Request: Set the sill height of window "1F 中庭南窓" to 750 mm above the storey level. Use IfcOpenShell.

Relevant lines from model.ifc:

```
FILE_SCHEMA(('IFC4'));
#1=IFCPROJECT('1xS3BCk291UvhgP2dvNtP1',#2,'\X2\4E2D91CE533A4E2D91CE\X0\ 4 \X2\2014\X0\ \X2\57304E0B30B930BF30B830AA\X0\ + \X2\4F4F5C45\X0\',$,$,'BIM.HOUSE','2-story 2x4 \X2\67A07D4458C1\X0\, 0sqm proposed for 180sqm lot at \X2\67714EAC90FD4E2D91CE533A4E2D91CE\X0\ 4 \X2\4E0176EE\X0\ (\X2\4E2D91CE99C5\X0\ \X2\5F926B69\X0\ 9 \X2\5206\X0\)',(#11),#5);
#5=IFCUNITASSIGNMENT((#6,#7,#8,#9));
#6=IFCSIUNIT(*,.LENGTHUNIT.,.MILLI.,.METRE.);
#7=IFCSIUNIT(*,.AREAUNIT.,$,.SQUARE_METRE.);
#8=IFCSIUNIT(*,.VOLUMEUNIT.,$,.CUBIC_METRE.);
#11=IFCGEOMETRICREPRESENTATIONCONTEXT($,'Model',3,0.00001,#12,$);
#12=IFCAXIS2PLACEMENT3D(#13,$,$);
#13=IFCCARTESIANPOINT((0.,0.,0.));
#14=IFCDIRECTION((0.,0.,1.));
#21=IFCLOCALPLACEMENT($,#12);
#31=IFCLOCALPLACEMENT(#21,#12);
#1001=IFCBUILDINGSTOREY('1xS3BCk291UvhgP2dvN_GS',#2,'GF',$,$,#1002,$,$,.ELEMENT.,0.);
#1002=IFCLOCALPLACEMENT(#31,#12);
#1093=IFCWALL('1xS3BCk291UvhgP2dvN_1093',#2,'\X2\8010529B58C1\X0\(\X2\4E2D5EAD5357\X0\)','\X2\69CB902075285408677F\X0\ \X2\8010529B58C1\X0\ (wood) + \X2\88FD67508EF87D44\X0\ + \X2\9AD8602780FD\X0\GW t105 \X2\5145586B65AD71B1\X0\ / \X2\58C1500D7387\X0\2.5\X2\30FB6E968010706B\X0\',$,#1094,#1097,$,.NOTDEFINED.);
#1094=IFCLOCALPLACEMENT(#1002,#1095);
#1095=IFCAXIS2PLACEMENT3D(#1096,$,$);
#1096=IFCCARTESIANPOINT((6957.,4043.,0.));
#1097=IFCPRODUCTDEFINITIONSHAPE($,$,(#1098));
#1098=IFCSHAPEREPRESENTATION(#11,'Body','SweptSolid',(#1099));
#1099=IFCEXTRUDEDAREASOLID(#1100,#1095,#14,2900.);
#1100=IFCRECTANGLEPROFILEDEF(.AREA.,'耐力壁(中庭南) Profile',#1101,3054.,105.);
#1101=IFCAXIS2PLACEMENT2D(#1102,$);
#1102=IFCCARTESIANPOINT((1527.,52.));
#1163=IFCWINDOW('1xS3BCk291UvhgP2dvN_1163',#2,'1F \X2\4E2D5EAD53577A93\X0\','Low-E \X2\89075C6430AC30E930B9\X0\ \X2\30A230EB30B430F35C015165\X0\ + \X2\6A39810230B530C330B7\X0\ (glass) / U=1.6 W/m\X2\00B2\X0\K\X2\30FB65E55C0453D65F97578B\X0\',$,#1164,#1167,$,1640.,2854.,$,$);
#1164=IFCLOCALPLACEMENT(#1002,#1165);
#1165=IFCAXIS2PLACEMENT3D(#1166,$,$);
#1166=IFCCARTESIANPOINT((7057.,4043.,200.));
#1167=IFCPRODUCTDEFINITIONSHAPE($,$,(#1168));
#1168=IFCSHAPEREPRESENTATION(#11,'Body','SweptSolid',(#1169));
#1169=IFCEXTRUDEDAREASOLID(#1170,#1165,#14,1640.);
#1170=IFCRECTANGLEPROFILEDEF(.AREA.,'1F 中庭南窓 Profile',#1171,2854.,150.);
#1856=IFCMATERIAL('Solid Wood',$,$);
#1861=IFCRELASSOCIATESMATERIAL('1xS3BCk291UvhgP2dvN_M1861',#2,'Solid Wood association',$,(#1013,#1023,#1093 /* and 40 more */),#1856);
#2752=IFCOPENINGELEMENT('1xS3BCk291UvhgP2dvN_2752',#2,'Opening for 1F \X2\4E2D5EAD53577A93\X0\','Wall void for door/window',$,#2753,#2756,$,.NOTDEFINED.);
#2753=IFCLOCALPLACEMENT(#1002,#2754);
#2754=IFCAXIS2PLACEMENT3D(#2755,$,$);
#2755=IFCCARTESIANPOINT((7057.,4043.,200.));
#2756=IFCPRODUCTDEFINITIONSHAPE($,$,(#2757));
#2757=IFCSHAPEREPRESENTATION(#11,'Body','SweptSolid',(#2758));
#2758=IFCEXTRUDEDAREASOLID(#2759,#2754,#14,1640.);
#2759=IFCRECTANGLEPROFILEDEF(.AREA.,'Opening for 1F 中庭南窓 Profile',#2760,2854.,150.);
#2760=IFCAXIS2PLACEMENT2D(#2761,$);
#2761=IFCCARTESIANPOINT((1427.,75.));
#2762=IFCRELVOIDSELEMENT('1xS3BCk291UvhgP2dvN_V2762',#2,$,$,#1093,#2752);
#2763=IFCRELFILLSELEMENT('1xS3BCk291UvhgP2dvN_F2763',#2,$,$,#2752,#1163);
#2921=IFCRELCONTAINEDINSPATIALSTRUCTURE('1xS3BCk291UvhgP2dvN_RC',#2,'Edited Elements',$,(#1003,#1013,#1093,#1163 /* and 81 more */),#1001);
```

```python
import numpy as np
import ifcopenshell
import ifcopenshell.api.geometry
import ifcopenshell.geom
import ifcopenshell.util.element
import ifcopenshell.util.placement
import ifcopenshell.util.shape
import ifcopenshell.util.unit

model = ifcopenshell.open("model.ifc")
unit_scale = ifcopenshell.util.unit.calculate_unit_scale(model)

window = model.by_id(1163)
opening = window.FillsVoids[0].RelatingOpeningElement
storey = ifcopenshell.util.element.get_container(window, ifc_class="IfcBuildingStorey")
level = ifcopenshell.util.placement.get_local_placement(storey.ObjectPlacement)[2, 3]

# The opening's origin need not be at the sill, so measure its lowest point.
shape = ifcopenshell.geom.create_shape(ifcopenshell.geom.settings(), opening)
bottom = ifcopenshell.util.shape.get_shape_bottom_elevation(shape, shape.geometry) / unit_scale
dz = level + 0.75 / unit_scale - bottom

shift = np.array([0.0, 0.0, dz])
# The window is not placed relative to its opening, so move both.
for product in (opening, window):
    matrix = ifcopenshell.util.placement.get_local_placement(product.ObjectPlacement)
    matrix[:3, 3] += shift
    ifcopenshell.api.geometry.edit_object_placement(model, product=product, matrix=matrix, is_si=False)

print(f"moved by {dz * unit_scale:+.3f} m")

model.write("model_v2.ifc")
```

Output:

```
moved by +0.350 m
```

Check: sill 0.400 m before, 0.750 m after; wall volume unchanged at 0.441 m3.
